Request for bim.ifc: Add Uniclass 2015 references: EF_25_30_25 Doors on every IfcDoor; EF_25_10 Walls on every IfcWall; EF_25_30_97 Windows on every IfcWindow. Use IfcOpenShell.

First a look at what the model holds.

```python
import ifcopenshell

model = ifcopenshell.open("bim.ifc")
print(model.schema)
print("classifications:", [c.Name for c in model.by_type("IfcClassification")])
for ifc_class in ("IfcDoor", "IfcRoof", "IfcStair", "IfcWall", "IfcWindow"):
    print(ifc_class, len(model.by_type(ifc_class)))
```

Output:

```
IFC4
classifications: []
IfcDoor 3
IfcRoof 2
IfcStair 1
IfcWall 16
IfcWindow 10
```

```python
import ifcopenshell
import ifcopenshell.api.classification

model = ifcopenshell.open("bim.ifc")

system = ifcopenshell.api.classification.add_classification(model, classification="Uniclass 2015")

codes = {
    "IfcDoor": ("EF_25_30_25", "Doors"),
    "IfcWall": ("EF_25_10", "Walls"),
    "IfcWindow": ("EF_25_30_97", "Windows"),
}
for ifc_class, (code, name) in codes.items():
    products = model.by_type(ifc_class)
    ifcopenshell.api.classification.add_reference(
        model, products=products, classification=system, identification=code, name=name
    )
    print(code, len(products))

model.write("bim_v2.ifc")
```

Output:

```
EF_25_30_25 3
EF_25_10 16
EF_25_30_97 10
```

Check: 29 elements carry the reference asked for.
